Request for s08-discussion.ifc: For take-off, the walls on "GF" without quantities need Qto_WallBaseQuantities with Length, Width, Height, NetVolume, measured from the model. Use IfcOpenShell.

First a look at what the model holds.

```python
import ifcopenshell
import ifcopenshell.util.element
import ifcopenshell.util.unit

model = ifcopenshell.open("s08-discussion.ifc")
print(model.schema)
for unit_type in ("LENGTHUNIT", "AREAUNIT", "VOLUMEUNIT"):
    print(unit_type, ifcopenshell.util.unit.calculate_unit_scale(model, unit_type))
storey = next(s for s in model.by_type("IfcBuildingStorey") if s.Name == "GF")
walls = [e for e in ifcopenshell.util.element.get_decomposition(storey) if e.is_a("IfcWall")]
for e in sorted(walls, key=lambda e: e.id()):
    print(e.id(), e.is_a(), e.Name, list(ifcopenshell.util.element.get_psets(e, qtos_only=True)), sep=" | ")
```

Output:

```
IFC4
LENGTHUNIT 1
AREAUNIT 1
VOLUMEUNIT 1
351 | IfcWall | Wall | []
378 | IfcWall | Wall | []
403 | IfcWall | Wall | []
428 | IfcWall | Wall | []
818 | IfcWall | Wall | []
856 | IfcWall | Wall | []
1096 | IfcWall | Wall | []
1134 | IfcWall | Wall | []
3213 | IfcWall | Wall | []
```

```python
import ifcopenshell
import ifcopenshell.api.pset
import ifcopenshell.geom
import ifcopenshell.util.element
import ifcopenshell.util.shape
import ifcopenshell.util.unit

model = ifcopenshell.open("s08-discussion.ifc")
unit_scale = ifcopenshell.util.unit.calculate_unit_scale(model)
volume_scale = ifcopenshell.util.unit.calculate_unit_scale(model, "VOLUMEUNIT")
settings = ifcopenshell.geom.settings()

storey = next(s for s in model.by_type("IfcBuildingStorey") if s.Name == "GF")
walls = [e for e in ifcopenshell.util.element.get_decomposition(storey) if e.is_a("IfcWall")]

for e in sorted(walls, key=lambda e: e.id()):
    if ifcopenshell.util.element.get_psets(e, qtos_only=True, should_inherit=False):
        continue
    # Geometry comes back in metres, in the element's own axes.
    shape = ifcopenshell.geom.create_shape(settings, e)
    values = {
        "Length": ifcopenshell.util.shape.get_x(shape.geometry) / unit_scale,
        "Width": ifcopenshell.util.shape.get_y(shape.geometry) / unit_scale,
        "Height": ifcopenshell.util.shape.get_z(shape.geometry) / unit_scale,
        "NetVolume": ifcopenshell.util.shape.get_volume(shape.geometry) / volume_scale,
    }
    qto = ifcopenshell.api.pset.add_qto(model, product=e, name="Qto_WallBaseQuantities")
    ifcopenshell.api.pset.edit_qto(model, qto=qto, properties=values)
    print(e.id(), {k: round(v, 3) for k, v in values.items()})

model.write("s08-discussion_rev.ifc")
```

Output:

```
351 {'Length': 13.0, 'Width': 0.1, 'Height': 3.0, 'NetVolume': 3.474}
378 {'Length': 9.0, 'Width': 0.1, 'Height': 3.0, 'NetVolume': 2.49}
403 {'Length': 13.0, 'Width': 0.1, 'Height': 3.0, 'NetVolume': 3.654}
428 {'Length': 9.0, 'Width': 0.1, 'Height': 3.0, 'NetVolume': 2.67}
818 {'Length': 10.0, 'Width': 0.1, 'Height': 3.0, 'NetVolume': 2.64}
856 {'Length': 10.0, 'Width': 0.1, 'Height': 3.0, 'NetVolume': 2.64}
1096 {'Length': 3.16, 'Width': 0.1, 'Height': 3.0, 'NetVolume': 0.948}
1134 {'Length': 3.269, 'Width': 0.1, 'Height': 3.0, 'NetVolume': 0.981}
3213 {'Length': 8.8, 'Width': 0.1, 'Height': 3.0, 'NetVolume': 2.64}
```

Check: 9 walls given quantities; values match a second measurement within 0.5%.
